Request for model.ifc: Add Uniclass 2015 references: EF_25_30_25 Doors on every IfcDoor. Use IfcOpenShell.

First a look at what the model holds.

```python
import ifcopenshell

model = ifcopenshell.open("model.ifc")
print(model.schema)
print("classifications:", [c.Name for c in model.by_type("IfcClassification")])
for ifc_class in ("IfcDoor", "IfcRoof", "IfcStair", "IfcWall", "IfcWindow"):
    print(ifc_class, len(model.by_type(ifc_class)))
```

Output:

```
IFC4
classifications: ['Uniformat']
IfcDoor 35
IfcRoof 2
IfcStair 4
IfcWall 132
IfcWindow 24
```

```python
import ifcopenshell
import ifcopenshell.api.classification

model = ifcopenshell.open("model.ifc")

system = ifcopenshell.api.classification.add_classification(model, classification="Uniclass 2015")

codes = {
    "IfcDoor": ("EF_25_30_25", "Doors"),
}
for ifc_class, (code, name) in codes.items():
    products = model.by_type(ifc_class)
    ifcopenshell.api.classification.add_reference(
        model, products=products, classification=system, identification=code, name=name
    )
    print(code, len(products))

model.write("model-out.ifc")
```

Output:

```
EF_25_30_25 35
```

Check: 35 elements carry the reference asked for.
